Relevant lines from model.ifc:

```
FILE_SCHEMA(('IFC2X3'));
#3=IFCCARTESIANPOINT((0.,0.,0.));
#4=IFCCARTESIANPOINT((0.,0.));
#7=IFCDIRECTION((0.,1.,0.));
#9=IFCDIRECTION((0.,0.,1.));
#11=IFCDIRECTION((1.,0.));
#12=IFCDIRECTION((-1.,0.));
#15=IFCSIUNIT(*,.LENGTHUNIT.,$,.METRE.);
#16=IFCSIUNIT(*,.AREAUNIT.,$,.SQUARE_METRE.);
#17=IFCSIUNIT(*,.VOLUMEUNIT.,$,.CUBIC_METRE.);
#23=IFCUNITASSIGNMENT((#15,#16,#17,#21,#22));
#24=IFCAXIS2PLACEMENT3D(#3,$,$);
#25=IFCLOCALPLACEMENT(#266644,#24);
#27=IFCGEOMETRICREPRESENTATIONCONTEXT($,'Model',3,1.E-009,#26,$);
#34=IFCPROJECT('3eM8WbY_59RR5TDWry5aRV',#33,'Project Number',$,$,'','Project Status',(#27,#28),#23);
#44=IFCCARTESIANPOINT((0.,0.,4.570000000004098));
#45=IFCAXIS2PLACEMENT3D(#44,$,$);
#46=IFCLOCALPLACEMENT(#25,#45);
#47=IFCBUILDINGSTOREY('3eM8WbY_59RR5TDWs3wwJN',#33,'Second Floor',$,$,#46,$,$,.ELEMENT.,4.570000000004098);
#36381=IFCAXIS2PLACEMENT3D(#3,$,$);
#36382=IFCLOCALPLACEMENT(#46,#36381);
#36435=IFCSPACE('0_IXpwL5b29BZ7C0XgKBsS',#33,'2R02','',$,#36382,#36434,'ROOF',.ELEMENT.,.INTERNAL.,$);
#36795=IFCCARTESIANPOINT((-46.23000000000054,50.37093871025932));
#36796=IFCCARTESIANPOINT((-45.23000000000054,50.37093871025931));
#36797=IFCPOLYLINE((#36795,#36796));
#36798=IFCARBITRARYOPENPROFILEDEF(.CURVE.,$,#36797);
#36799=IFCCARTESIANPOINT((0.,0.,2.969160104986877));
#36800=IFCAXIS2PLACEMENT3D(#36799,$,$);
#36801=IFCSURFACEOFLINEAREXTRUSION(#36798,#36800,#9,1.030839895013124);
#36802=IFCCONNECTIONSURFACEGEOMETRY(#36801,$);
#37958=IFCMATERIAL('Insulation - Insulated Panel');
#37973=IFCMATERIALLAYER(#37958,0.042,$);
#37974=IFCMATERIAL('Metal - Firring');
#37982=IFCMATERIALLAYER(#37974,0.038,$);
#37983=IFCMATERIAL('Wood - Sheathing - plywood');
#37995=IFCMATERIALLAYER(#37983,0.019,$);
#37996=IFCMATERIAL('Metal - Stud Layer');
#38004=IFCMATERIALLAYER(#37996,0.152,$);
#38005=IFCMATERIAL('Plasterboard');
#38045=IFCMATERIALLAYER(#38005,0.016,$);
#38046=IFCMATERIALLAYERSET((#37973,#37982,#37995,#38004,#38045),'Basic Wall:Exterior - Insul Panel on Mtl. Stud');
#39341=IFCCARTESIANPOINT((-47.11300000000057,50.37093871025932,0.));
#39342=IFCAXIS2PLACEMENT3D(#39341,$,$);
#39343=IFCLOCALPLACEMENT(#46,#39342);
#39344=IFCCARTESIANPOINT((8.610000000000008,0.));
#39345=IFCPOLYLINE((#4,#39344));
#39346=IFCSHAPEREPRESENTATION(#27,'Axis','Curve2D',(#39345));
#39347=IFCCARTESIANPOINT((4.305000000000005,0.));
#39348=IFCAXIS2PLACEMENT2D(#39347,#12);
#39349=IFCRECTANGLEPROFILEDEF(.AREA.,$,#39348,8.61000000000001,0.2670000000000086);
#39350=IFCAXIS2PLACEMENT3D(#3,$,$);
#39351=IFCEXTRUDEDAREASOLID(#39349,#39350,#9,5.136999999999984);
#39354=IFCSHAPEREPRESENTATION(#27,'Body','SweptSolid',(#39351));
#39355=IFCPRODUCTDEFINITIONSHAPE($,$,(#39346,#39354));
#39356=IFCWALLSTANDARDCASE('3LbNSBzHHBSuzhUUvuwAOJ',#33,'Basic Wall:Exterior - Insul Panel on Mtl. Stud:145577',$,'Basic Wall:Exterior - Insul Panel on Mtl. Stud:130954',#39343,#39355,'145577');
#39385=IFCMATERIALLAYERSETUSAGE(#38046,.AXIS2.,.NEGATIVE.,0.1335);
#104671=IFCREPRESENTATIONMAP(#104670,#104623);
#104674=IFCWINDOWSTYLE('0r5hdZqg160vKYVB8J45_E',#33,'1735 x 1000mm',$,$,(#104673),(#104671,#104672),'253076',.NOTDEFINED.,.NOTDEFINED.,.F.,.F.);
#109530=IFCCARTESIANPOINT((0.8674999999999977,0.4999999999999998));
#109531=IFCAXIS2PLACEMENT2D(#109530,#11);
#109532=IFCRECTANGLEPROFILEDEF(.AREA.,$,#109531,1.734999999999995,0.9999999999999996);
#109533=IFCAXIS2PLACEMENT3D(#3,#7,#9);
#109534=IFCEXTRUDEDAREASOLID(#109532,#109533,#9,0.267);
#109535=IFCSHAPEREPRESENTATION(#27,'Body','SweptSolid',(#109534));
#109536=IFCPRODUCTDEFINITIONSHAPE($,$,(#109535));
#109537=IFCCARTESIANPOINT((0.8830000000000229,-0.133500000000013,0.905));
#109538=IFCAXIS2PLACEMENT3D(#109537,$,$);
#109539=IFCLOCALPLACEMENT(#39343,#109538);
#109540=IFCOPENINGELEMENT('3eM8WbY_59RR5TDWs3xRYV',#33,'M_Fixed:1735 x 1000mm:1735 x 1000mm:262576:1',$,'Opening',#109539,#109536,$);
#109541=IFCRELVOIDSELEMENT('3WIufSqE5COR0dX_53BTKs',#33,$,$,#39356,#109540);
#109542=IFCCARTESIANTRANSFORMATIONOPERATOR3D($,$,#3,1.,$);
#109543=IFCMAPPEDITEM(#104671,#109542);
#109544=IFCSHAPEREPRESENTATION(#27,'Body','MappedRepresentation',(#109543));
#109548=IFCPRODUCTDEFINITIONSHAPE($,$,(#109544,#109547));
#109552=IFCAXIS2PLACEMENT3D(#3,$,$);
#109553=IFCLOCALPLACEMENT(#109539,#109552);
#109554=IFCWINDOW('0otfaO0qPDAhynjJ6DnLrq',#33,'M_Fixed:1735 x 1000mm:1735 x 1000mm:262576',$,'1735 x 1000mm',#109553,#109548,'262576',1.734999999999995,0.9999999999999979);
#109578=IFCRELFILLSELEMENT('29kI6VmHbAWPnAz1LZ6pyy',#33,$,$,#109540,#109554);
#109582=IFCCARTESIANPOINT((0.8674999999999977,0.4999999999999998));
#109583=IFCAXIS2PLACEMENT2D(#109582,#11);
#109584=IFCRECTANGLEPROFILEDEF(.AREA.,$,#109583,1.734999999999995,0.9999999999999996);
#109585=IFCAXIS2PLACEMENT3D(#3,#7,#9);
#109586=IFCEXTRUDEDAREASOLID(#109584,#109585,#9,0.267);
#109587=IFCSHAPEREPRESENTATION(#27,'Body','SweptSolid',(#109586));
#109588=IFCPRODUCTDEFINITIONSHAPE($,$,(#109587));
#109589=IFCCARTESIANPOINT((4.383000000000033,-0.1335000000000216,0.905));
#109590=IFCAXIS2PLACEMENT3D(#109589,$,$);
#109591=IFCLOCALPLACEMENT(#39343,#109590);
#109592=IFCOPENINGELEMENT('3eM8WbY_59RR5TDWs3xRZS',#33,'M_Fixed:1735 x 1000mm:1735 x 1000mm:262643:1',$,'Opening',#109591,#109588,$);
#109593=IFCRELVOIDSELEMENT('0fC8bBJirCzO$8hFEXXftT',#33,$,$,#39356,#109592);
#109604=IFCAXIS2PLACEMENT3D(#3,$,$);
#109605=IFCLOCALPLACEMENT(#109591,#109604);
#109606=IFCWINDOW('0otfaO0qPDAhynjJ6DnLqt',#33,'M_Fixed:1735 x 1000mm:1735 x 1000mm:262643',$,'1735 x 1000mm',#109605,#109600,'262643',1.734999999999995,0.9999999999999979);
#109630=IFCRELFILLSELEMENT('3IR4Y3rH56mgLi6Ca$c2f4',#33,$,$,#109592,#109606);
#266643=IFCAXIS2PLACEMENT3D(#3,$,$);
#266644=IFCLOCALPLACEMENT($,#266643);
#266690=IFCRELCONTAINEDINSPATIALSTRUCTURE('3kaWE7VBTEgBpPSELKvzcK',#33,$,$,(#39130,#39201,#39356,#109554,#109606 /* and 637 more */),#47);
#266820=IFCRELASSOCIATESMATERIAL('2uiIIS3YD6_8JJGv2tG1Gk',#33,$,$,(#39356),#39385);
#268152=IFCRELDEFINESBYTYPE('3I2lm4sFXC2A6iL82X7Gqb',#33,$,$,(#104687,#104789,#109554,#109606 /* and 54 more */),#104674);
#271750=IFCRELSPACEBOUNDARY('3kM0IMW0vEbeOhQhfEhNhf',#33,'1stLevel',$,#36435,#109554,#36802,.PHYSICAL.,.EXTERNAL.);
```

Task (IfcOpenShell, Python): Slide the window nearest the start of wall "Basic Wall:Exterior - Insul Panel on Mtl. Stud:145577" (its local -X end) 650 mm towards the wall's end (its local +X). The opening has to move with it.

```python
import numpy as np
import ifcopenshell
import ifcopenshell.api.geometry
import ifcopenshell.util.placement

model = ifcopenshell.open("model.ifc")

window = model.by_guid("0otfaO0qPDAhynjJ6DnLrq")
opening = window.FillsVoids[0].RelatingOpeningElement
wall = opening.VoidsElements[0].RelatingBuildingElement

wall_matrix = ifcopenshell.util.placement.get_local_placement(wall.ObjectPlacement)
shift = wall_matrix[:3, 0] * 0.65
before = ifcopenshell.util.placement.get_local_placement(window.ObjectPlacement)[:3, 3].copy()

# The window is placed relative to its opening, so it follows when the opening moves.
matrix = ifcopenshell.util.placement.get_local_placement(opening.ObjectPlacement)
matrix[:3, 3] += shift
ifcopenshell.api.geometry.edit_object_placement(
    model, product=opening, matrix=matrix, is_si=False, should_transform_children=True
)

# Space boundary surfaces are stored in each space's coordinates; move them too.
for rel in window.ProvidesBoundaries:
    if not rel.ConnectionGeometry:
        continue
    surface = rel.ConnectionGeometry.SurfaceOnRelatingElement
    space_matrix = ifcopenshell.util.placement.get_local_placement(rel.RelatingSpace.ObjectPlacement)
    point = np.array(surface.Position.Location.Coordinates) + space_matrix[:3, :3].T @ shift
    surface.Position = model.createIfcAxis2Placement3D(
        model.createIfcCartesianPoint(point.tolist()), surface.Position.Axis, surface.Position.RefDirection
    )

after = ifcopenshell.util.placement.get_local_placement(window.ObjectPlacement)[:3, 3]
print("window moved by", (after - before).round(3) + 0.0)

model.write("model-out.ifc")
```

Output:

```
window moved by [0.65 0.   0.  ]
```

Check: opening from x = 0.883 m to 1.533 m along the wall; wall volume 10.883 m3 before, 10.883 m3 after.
